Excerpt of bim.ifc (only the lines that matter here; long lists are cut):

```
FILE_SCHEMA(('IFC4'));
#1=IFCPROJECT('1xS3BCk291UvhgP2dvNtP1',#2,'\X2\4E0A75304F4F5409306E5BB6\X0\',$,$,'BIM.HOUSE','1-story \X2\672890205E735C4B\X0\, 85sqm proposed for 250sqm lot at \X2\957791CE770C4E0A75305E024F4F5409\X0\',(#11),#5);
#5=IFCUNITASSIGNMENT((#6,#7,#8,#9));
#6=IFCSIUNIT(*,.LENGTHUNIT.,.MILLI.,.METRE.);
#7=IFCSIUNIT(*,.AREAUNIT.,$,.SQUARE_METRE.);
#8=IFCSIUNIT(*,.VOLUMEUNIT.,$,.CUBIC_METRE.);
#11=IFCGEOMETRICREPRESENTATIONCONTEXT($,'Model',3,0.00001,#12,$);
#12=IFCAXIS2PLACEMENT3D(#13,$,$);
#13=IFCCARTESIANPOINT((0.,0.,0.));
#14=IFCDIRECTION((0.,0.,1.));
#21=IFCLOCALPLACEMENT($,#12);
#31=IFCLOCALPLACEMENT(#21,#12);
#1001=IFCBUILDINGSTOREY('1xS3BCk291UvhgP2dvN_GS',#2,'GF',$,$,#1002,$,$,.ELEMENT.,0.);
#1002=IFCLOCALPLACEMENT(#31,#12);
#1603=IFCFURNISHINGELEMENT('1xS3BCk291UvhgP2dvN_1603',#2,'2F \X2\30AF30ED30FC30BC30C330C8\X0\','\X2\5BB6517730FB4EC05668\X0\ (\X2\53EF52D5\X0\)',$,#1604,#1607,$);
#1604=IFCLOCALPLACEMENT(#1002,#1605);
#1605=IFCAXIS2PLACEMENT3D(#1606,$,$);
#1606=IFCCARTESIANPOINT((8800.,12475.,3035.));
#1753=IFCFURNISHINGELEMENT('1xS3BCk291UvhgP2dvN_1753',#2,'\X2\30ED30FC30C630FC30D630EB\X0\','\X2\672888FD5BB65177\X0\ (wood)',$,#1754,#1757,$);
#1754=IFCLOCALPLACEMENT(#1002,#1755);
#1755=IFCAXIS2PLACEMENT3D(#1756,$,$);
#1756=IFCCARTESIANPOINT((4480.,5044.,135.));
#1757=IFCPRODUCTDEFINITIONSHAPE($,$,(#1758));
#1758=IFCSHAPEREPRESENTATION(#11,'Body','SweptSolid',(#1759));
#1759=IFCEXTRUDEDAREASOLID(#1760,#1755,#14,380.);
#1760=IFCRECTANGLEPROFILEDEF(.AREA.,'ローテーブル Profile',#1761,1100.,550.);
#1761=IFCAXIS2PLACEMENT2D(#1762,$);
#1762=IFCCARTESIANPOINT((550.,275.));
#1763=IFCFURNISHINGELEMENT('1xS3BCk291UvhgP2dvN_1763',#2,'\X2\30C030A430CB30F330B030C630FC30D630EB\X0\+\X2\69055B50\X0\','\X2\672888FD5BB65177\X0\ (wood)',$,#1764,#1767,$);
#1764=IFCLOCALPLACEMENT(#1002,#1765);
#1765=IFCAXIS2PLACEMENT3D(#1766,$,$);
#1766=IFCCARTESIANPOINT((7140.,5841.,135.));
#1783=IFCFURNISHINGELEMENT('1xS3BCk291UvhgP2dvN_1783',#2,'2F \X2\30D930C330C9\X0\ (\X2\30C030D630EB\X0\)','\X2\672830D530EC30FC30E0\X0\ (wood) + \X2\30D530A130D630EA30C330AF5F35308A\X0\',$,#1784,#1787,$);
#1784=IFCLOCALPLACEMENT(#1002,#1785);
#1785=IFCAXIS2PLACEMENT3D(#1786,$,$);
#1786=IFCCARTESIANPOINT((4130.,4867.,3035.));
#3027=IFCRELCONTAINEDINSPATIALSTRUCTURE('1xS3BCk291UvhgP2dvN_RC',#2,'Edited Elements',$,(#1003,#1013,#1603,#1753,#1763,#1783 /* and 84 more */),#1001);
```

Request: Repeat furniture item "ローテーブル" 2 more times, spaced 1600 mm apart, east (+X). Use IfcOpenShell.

```python
import numpy as np
import ifcopenshell
import ifcopenshell.api.geometry
import ifcopenshell.api.root
import ifcopenshell.util.element
import ifcopenshell.util.placement

model = ifcopenshell.open("bim.ifc")


def reuse_history(source, copy):
    """copy_class also copies each property set's owner history, people and application; keep the originals."""
    for rel in copy.IsDefinedBy:
        if rel.is_a("IfcRelDefinesByProperties") and (history := rel.RelatingPropertyDefinition.OwnerHistory):
            rel.RelatingPropertyDefinition.OwnerHistory = source.OwnerHistory
            ifcopenshell.util.element.remove_deep2(model, history)


source = model.by_guid("1xS3BCk291UvhgP2dvN_1753")
base = ifcopenshell.util.placement.get_local_placement(source.ObjectPlacement)
step = np.array([1.0, 0.0, 0.0]) * 1600.0

for i in range(1, 3):
    copy = ifcopenshell.api.root.copy_class(model, product=source)
    copy.Representation = ifcopenshell.util.element.copy_deep(
        model, source.Representation, exclude=["IfcGeometricRepresentationContext", "IfcRepresentationMap"]
    )
    reuse_history(source, copy)
    matrix = base.copy()
    matrix[:3, 3] += i * step
    print("added at", matrix[:3, 3].round(3) + 0.0)
    ifcopenshell.api.geometry.edit_object_placement(model, product=copy, matrix=matrix, is_si=False)

model.write("bim_updated.ifc")
```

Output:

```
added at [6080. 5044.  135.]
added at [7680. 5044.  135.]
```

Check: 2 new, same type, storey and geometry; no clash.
